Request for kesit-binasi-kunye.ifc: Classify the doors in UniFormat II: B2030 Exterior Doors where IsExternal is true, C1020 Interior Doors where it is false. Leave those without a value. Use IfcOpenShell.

First a look at what the model holds.

```python
import ifcopenshell
import ifcopenshell.util.element

model = ifcopenshell.open("kesit-binasi-kunye.ifc")
print(model.schema)
print("classifications:", [c.Name for c in model.by_type("IfcClassification")])
values = [ifcopenshell.util.element.get_pset(e, "Pset_DoorCommon", "IsExternal") for e in model.by_type("IfcDoor")]
for value in (True, False, None):
    print("IsExternal", value, values.count(value))
```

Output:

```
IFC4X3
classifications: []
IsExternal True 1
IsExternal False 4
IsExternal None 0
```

```python
import ifcopenshell
import ifcopenshell.api.classification
import ifcopenshell.util.element

model = ifcopenshell.open("kesit-binasi-kunye.ifc")

system = ifcopenshell.api.classification.add_classification(model, classification="UniFormat II")

doors = model.by_type("IfcDoor")
external = {e: ifcopenshell.util.element.get_pset(e, "Pset_DoorCommon", "IsExternal") for e in doors}
for flag, code, name in ((True, "B2030", "Exterior Doors"), (False, "C1020", "Interior Doors")):
    products = [e for e in doors if external[e] is flag]
    ifcopenshell.api.classification.add_reference(
        model, products=products, classification=system, identification=code, name=name
    )
    print(code, len(products))

model.write("kesit-binasi-kunye_rev.ifc")
```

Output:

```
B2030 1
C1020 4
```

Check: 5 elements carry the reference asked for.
